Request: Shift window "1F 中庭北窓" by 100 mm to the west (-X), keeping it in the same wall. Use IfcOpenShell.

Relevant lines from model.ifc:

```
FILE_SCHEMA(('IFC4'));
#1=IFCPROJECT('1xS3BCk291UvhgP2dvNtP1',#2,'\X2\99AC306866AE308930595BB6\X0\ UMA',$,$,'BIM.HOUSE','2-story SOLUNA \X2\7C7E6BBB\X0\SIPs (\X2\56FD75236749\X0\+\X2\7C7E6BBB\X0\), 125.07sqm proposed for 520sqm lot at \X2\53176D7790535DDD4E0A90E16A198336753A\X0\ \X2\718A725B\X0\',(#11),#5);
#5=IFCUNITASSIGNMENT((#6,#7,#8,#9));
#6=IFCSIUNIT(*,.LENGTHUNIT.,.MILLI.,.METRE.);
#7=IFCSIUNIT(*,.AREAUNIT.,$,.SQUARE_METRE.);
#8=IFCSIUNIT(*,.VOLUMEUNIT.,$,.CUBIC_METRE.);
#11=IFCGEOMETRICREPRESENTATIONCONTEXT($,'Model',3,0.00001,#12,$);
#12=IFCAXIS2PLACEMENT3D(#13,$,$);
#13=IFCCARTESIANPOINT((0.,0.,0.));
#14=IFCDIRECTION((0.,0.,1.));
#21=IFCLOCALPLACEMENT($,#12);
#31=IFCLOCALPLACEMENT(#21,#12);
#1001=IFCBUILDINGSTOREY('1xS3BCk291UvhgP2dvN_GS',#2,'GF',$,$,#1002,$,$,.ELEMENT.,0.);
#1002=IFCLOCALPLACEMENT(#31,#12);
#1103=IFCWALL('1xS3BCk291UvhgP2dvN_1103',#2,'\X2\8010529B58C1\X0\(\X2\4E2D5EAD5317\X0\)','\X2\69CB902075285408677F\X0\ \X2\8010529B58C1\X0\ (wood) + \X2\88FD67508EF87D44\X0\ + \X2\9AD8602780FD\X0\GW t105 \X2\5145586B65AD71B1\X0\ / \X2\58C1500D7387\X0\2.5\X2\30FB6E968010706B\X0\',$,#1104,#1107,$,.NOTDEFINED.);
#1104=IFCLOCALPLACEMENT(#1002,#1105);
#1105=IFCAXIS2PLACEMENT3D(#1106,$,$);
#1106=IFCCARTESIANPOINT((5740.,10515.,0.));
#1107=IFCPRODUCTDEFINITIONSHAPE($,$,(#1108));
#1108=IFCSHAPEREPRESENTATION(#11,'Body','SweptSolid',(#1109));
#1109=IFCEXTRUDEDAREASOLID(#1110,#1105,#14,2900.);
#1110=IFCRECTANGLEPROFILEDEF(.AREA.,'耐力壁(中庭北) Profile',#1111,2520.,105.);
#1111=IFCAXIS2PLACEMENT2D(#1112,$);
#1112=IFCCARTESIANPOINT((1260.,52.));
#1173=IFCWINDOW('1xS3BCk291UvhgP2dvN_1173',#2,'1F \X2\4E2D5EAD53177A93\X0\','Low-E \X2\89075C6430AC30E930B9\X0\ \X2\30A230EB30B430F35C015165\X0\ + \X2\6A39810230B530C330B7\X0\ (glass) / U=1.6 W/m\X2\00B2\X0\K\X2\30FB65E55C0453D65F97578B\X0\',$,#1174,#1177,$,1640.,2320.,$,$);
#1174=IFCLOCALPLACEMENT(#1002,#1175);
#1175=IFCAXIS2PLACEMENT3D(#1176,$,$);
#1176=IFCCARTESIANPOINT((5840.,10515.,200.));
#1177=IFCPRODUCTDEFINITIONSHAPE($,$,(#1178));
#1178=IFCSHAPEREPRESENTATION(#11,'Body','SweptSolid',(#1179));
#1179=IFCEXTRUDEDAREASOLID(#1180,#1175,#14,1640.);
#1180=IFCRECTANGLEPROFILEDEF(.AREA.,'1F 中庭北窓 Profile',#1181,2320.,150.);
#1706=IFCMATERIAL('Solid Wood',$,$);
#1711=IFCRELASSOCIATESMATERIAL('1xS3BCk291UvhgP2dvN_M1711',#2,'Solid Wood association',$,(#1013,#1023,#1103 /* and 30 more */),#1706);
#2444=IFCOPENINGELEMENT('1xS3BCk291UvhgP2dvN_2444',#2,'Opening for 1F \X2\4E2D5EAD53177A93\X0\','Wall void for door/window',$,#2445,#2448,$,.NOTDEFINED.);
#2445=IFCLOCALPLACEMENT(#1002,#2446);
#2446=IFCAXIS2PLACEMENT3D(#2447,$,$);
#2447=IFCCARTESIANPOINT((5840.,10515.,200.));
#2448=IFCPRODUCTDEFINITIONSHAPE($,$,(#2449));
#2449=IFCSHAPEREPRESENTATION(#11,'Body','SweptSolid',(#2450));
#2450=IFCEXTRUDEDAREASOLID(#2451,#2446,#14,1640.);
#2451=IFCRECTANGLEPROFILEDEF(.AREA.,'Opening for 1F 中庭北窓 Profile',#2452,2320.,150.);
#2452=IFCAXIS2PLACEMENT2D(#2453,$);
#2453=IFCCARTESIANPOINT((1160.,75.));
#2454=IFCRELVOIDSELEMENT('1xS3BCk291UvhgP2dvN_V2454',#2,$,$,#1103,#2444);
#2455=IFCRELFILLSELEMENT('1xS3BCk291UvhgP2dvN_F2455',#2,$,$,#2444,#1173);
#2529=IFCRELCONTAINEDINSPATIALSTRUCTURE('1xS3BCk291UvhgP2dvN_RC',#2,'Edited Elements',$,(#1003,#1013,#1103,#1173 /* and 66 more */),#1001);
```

```python
import ifcopenshell
import ifcopenshell.api.geometry
import ifcopenshell.util.placement
import ifcopenshell.util.unit

model = ifcopenshell.open("model.ifc")
unit_scale = ifcopenshell.util.unit.calculate_unit_scale(model)

window = model.by_guid("1xS3BCk291UvhgP2dvN_1173")
opening = window.FillsVoids[0].RelatingOpeningElement
wall = opening.VoidsElements[0].RelatingBuildingElement

wall_matrix = ifcopenshell.util.placement.get_local_placement(wall.ObjectPlacement)
shift = wall_matrix[:3, 0] * -0.1 / unit_scale
before = ifcopenshell.util.placement.get_local_placement(window.ObjectPlacement)[:3, 3].copy()

# The window is not placed relative to its opening, so move both.
for product in (opening, window):
    matrix = ifcopenshell.util.placement.get_local_placement(product.ObjectPlacement)
    matrix[:3, 3] += shift
    ifcopenshell.api.geometry.edit_object_placement(model, product=product, matrix=matrix, is_si=False)

after = ifcopenshell.util.placement.get_local_placement(window.ObjectPlacement)[:3, 3]
print("window moved by", (after - before).round(3) + 0.0)

model.write("model_edited.ifc")
```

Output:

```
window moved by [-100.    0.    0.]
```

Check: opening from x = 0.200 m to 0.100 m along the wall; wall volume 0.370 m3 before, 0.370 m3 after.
